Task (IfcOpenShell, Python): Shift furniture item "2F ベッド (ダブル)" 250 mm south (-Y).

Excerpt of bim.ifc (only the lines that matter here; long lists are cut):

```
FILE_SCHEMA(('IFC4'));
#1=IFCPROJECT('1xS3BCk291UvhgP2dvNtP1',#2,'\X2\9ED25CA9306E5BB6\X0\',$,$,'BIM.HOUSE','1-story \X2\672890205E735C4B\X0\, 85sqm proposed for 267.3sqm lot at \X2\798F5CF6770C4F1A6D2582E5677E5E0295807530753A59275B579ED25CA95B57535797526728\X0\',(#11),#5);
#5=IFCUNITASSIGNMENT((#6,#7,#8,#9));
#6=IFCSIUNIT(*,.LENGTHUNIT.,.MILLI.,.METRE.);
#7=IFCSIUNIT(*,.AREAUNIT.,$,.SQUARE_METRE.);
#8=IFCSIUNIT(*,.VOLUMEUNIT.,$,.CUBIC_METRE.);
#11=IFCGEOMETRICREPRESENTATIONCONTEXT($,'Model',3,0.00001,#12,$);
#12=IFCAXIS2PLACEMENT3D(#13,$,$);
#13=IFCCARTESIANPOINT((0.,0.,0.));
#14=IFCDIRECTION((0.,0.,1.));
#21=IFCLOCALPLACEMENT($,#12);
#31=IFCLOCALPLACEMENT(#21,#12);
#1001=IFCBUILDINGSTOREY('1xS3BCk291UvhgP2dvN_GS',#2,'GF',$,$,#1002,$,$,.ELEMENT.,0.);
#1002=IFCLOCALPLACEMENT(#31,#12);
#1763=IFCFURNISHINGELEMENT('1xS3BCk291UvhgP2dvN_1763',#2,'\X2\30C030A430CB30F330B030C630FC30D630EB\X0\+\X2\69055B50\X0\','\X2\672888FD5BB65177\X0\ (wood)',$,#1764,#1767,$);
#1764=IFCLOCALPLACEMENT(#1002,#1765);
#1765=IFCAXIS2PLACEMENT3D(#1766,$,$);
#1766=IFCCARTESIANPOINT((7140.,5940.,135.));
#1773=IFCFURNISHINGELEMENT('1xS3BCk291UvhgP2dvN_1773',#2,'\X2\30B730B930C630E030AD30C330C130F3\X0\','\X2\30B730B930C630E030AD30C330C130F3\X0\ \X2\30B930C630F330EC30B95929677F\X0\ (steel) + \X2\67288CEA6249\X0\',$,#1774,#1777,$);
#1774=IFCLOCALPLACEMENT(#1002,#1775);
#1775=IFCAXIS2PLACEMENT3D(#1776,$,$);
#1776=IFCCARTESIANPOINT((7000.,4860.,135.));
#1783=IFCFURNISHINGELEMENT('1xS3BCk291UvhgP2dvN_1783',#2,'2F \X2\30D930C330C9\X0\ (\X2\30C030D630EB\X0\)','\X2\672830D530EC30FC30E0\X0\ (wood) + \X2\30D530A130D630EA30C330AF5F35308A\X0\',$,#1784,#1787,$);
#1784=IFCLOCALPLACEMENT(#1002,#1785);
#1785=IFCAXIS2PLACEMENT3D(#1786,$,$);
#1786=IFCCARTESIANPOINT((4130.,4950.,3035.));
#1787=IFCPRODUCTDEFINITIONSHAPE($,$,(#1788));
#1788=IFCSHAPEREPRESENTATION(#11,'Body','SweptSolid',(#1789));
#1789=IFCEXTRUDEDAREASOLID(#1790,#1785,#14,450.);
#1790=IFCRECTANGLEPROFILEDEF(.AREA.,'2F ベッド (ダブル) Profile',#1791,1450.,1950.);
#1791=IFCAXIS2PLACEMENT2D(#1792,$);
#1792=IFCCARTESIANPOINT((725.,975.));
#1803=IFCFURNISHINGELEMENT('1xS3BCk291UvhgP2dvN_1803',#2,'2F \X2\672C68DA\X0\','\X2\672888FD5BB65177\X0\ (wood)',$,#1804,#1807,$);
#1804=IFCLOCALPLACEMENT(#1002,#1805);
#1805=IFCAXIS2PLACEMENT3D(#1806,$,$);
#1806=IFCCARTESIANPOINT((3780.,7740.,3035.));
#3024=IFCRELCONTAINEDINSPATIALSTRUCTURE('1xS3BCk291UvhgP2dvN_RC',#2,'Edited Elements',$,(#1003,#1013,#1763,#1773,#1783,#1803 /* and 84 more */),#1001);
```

```python
import ifcopenshell
import ifcopenshell.api.geometry
import ifcopenshell.util.placement
import ifcopenshell.util.unit

model = ifcopenshell.open("bim.ifc")
unit_scale = ifcopenshell.util.unit.calculate_unit_scale(model)

item = model.by_id(1783)
matrix = ifcopenshell.util.placement.get_local_placement(item.ObjectPlacement)
matrix[1, 3] -= 0.25 / unit_scale
ifcopenshell.api.geometry.edit_object_placement(model, product=item, matrix=matrix, is_si=False)

print(ifcopenshell.util.placement.get_local_placement(item.ObjectPlacement).round(3) + 0.0)

model.write("bim_edited.ifc")
```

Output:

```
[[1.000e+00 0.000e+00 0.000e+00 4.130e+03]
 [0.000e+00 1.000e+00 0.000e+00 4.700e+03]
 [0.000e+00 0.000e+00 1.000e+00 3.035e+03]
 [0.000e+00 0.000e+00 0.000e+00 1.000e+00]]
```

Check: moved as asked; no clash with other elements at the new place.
